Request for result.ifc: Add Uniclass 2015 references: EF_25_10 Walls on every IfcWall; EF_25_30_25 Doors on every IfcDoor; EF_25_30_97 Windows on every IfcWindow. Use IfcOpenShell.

First a look at what the model holds.

```python
import ifcopenshell

model = ifcopenshell.open("result.ifc")
print(model.schema)
print("classifications:", [c.Name for c in model.by_type("IfcClassification")])
for ifc_class in ("IfcDoor", "IfcRoof", "IfcStair", "IfcWall", "IfcWindow"):
    print(ifc_class, len(model.by_type(ifc_class)))
```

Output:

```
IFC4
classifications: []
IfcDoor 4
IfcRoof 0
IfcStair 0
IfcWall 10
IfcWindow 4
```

```python
import ifcopenshell
import ifcopenshell.api.classification

model = ifcopenshell.open("result.ifc")

system = ifcopenshell.api.classification.add_classification(model, classification="Uniclass 2015")

codes = {
    "IfcWall": ("EF_25_10", "Walls"),
    "IfcDoor": ("EF_25_30_25", "Doors"),
    "IfcWindow": ("EF_25_30_97", "Windows"),
}
for ifc_class, (code, name) in codes.items():
    products = model.by_type(ifc_class)
    ifcopenshell.api.classification.add_reference(
        model, products=products, classification=system, identification=code, name=name
    )
    print(code, len(products))

model.write("result_edited.ifc")
```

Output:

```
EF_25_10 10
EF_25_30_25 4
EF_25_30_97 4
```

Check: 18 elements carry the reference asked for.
